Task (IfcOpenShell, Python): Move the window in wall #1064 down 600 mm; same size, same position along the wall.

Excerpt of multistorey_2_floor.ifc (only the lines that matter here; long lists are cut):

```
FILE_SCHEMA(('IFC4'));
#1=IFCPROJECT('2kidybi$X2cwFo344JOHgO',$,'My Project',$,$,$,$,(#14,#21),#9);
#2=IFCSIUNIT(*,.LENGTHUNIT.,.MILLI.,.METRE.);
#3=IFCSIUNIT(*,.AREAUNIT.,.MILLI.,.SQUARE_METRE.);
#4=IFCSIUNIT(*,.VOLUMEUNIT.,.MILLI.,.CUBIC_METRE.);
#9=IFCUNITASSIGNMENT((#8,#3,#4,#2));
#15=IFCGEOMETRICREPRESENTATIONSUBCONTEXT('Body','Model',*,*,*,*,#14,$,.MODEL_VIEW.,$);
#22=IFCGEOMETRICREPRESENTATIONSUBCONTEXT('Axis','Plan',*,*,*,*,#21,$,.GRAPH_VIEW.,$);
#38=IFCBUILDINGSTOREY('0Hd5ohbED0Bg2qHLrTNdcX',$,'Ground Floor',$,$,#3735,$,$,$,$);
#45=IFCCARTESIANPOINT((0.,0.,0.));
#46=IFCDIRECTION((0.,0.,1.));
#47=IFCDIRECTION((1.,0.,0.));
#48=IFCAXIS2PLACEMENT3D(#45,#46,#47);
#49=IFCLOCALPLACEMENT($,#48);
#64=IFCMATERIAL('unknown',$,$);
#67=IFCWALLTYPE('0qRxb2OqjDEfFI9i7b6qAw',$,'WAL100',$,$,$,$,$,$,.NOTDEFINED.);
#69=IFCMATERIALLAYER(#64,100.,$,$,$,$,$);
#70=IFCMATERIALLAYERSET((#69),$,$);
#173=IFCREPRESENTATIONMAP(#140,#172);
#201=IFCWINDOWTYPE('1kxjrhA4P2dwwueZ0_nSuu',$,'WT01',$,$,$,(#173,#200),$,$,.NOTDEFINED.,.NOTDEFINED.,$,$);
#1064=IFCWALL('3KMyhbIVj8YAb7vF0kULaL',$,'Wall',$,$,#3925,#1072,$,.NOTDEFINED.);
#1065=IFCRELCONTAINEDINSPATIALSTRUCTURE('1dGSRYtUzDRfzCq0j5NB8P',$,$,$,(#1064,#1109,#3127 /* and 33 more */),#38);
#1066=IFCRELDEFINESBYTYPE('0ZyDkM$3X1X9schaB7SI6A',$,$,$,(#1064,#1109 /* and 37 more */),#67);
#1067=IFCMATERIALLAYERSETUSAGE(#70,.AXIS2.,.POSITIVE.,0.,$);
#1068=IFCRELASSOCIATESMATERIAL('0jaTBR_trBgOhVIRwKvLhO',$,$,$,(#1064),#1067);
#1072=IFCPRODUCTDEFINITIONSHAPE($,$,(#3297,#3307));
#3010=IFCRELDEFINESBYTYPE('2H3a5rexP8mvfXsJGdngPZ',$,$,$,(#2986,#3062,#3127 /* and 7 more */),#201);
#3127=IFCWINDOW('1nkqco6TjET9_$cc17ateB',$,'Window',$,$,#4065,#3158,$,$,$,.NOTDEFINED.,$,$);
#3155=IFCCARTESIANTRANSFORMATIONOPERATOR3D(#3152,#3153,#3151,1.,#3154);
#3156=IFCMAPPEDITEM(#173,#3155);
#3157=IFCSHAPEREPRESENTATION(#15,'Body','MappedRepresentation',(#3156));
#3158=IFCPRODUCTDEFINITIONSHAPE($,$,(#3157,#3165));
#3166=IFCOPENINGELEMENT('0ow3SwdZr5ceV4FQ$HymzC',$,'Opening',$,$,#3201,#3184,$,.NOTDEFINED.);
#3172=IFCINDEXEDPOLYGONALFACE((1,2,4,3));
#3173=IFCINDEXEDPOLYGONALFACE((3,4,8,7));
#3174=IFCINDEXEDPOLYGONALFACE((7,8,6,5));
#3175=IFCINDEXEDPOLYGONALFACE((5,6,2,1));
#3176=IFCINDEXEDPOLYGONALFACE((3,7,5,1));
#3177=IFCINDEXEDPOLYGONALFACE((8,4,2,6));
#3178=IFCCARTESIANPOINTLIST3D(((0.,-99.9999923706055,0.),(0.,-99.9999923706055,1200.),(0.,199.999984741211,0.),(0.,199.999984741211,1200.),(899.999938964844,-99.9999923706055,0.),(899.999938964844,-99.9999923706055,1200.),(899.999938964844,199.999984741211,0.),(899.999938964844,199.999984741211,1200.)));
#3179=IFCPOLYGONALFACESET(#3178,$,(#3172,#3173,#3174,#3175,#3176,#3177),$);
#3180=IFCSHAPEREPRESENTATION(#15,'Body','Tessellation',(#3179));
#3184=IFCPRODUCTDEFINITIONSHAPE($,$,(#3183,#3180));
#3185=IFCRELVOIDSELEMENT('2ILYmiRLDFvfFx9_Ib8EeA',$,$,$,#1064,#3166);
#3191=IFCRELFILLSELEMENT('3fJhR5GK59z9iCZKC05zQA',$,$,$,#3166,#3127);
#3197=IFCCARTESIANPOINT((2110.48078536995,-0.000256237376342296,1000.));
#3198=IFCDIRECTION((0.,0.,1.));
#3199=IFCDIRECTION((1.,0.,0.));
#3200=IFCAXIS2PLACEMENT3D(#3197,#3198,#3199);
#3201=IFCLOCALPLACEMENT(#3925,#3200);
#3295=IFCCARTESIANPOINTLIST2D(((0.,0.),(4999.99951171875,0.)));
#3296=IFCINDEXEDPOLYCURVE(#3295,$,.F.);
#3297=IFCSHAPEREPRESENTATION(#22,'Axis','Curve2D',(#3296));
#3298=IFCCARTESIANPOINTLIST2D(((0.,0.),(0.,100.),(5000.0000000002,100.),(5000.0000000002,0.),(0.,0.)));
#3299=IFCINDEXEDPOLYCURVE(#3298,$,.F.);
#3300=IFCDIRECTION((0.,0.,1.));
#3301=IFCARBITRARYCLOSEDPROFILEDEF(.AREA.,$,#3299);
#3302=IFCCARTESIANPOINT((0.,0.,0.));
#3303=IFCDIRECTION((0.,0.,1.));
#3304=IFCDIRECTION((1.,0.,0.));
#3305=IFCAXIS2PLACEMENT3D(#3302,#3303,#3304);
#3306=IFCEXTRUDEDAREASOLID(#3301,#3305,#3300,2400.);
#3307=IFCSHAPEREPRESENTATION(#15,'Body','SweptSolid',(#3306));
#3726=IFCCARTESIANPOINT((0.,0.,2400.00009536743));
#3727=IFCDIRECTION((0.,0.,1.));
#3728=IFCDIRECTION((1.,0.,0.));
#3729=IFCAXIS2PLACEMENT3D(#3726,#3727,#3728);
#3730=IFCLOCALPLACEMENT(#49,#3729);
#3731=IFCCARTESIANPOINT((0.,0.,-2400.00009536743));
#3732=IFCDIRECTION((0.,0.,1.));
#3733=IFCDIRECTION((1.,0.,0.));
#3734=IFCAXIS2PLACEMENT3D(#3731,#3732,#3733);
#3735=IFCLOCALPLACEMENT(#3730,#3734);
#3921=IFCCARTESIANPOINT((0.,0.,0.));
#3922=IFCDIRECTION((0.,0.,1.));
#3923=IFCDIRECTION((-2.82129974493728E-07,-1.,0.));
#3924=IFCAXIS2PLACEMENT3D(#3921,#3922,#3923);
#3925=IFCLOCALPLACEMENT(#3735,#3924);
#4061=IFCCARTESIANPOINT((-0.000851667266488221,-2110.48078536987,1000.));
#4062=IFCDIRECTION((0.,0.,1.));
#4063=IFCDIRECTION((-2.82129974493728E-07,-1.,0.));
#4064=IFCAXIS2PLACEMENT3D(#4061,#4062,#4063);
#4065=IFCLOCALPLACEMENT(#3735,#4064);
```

```python
import numpy as np
import ifcopenshell
import ifcopenshell.api.geometry
import ifcopenshell.util.placement
import ifcopenshell.util.unit

model = ifcopenshell.open("multistorey_2_floor.ifc")
unit_scale = ifcopenshell.util.unit.calculate_unit_scale(model)

window = model.by_id(3127)
opening = window.FillsVoids[0].RelatingOpeningElement
dz = -0.6 / unit_scale

shift = np.array([0.0, 0.0, dz])
# The window is not placed relative to its opening, so move both.
for product in (opening, window):
    matrix = ifcopenshell.util.placement.get_local_placement(product.ObjectPlacement)
    matrix[:3, 3] += shift
    ifcopenshell.api.geometry.edit_object_placement(model, product=product, matrix=matrix, is_si=False)

print(f"moved by {dz * unit_scale:+.3f} m")

model.write("multistorey_2_floor_updated.ifc")
```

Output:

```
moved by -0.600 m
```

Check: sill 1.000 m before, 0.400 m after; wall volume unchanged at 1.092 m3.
